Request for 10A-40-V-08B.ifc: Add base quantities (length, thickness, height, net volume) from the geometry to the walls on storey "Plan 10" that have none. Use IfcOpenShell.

First a look at what the model holds.

```python
import ifcopenshell
import ifcopenshell.util.element
import ifcopenshell.util.unit

model = ifcopenshell.open("10A-40-V-08B.ifc")
print(model.schema)
for unit_type in ("LENGTHUNIT", "AREAUNIT", "VOLUMEUNIT"):
    print(unit_type, ifcopenshell.util.unit.calculate_unit_scale(model, unit_type))
storey = next(s for s in model.by_type("IfcBuildingStorey") if s.Name == "Plan 10")
walls = [e for e in ifcopenshell.util.element.get_decomposition(storey) if e.is_a("IfcWall")]
for e in sorted(walls, key=lambda e: e.id()):
    print(e.id(), e.is_a(), e.Name, list(ifcopenshell.util.element.get_psets(e, qtos_only=True)), sep=" | ")
```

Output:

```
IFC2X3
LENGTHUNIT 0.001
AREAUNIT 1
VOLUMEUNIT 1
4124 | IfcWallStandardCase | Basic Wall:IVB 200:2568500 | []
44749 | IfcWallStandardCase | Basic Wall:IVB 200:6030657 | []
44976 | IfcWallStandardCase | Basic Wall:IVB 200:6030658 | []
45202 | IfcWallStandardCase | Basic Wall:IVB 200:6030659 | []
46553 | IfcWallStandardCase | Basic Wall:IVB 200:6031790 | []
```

```python
import ifcopenshell
import ifcopenshell.api.pset
import ifcopenshell.geom
import ifcopenshell.util.element
import ifcopenshell.util.shape
import ifcopenshell.util.unit

model = ifcopenshell.open("10A-40-V-08B.ifc")
unit_scale = ifcopenshell.util.unit.calculate_unit_scale(model)
volume_scale = ifcopenshell.util.unit.calculate_unit_scale(model, "VOLUMEUNIT")
settings = ifcopenshell.geom.settings()

storey = next(s for s in model.by_type("IfcBuildingStorey") if s.Name == "Plan 10")
walls = [e for e in ifcopenshell.util.element.get_decomposition(storey) if e.is_a("IfcWall")]

for e in sorted(walls, key=lambda e: e.id()):
    if ifcopenshell.util.element.get_psets(e, qtos_only=True, should_inherit=False):
        continue
    # Geometry comes back in metres, in the element's own axes.
    shape = ifcopenshell.geom.create_shape(settings, e)
    values = {
        "Length": ifcopenshell.util.shape.get_x(shape.geometry) / unit_scale,
        "Width": ifcopenshell.util.shape.get_y(shape.geometry) / unit_scale,
        "Height": ifcopenshell.util.shape.get_z(shape.geometry) / unit_scale,
        "NetVolume": ifcopenshell.util.shape.get_volume(shape.geometry) / volume_scale,
    }
    qto = ifcopenshell.api.pset.add_qto(model, product=e, name="BaseQuantities")
    ifcopenshell.api.pset.edit_qto(model, qto=qto, properties=values)
    print(e.id(), {k: round(v, 3) for k, v in values.items()})

model.write("10A-40-V-08B_v2.ifc")
```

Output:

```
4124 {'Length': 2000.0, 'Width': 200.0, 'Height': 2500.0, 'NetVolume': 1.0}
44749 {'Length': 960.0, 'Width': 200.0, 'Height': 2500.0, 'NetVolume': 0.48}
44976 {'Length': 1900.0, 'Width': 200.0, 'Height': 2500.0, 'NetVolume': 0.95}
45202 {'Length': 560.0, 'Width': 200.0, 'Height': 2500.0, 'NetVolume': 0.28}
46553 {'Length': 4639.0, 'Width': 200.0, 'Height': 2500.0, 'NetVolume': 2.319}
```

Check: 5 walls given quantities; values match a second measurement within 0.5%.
